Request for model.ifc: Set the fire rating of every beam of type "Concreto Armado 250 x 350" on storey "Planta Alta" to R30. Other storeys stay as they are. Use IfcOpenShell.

First a look at what the model holds.

```python
import ifcopenshell
import ifcopenshell.util.element

model = ifcopenshell.open("model.ifc")
print(model.schema)
storey = next(s for s in model.by_type("IfcBuildingStorey") if s.Name == "Planta Alta")
beams = [e for e in ifcopenshell.util.element.get_decomposition(storey) if e.is_a("IfcBeam")]
seen = {}
for e in beams:
    element_type = ifcopenshell.util.element.get_type(e)
    key = (element_type.Name if element_type != e and element_type else None, ifcopenshell.util.element.get_pset(e, "Pset_BeamCommon", "FireRating"))
    seen[key] = seen.get(key, 0) + 1
for (name, value), count in sorted(seen.items(), key=str):
    print(count, "x", name, "|", value)
```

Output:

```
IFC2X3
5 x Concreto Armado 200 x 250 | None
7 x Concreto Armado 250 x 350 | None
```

```python
import ifcopenshell
import ifcopenshell.api.pset
import ifcopenshell.util.element

model = ifcopenshell.open("model.ifc")

storey = next(s for s in model.by_type("IfcBuildingStorey") if s.Name == "Planta Alta")
beams = [e for e in ifcopenshell.util.element.get_decomposition(storey) if e.is_a("IfcBeam")]

count = 0
for e in beams:
    element_type = ifcopenshell.util.element.get_type(e)
    if element_type in (None, e) or element_type.Name != "Concreto Armado 250 x 350":
        continue
    # add_pset returns the element's existing set when there is one.
    pset = ifcopenshell.api.pset.add_pset(model, product=e, name="Pset_BeamCommon")
    ifcopenshell.api.pset.edit_pset(model, pset=pset, properties={"FireRating": "R30"})
    count += 1

print(count, "beams updated")

model.write("model_rev.ifc")
```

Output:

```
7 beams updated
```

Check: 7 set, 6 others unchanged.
